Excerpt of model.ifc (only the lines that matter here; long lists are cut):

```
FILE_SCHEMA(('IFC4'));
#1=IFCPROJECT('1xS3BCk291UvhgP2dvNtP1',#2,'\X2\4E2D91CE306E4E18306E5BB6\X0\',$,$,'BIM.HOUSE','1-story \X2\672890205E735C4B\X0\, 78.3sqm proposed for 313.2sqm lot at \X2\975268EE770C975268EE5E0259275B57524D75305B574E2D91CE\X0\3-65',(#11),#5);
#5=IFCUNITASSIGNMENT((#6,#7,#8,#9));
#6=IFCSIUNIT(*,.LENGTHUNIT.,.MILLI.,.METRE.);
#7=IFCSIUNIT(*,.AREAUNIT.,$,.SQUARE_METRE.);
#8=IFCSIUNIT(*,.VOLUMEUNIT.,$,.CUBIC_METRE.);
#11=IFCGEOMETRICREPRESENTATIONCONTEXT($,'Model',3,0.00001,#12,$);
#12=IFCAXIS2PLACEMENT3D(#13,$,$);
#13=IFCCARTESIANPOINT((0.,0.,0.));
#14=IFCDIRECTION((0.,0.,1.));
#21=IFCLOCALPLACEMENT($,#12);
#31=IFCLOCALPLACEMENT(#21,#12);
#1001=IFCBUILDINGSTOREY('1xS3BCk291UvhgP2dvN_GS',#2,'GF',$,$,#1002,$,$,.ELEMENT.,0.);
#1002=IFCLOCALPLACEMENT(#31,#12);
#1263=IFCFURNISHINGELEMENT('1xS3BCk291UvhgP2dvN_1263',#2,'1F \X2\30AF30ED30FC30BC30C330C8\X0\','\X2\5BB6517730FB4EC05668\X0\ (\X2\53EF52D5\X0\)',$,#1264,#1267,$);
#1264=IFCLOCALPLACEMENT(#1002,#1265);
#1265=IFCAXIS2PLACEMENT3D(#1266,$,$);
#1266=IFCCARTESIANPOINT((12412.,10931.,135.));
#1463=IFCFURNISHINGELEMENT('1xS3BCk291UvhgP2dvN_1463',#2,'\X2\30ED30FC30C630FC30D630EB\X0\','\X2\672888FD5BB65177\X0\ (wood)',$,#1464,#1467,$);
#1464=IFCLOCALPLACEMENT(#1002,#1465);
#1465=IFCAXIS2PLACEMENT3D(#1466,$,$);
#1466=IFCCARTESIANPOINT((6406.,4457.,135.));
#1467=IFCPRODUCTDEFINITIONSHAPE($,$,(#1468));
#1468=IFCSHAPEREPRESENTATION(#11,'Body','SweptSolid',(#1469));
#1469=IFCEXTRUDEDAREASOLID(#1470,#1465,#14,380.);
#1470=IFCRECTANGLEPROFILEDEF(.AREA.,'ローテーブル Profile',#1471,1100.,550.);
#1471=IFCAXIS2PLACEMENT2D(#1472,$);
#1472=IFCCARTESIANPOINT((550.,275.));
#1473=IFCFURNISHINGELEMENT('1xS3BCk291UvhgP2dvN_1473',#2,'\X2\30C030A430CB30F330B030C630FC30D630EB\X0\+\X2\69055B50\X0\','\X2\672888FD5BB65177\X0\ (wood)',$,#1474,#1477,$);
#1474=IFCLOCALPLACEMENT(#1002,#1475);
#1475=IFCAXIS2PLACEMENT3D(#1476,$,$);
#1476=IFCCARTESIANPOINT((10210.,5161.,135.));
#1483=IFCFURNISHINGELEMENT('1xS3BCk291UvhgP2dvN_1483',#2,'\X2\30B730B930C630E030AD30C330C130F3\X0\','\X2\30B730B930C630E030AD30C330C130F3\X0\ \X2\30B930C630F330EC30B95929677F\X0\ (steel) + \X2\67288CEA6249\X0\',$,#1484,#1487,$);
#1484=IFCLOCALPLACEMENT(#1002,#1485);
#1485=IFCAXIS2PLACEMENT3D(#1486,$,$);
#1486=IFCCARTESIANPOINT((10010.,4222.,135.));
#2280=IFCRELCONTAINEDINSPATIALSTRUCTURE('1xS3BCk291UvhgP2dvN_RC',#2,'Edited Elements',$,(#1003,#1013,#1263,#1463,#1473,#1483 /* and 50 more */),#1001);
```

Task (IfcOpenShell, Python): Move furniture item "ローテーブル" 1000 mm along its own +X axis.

```python
import ifcopenshell
import ifcopenshell.api.geometry
import ifcopenshell.util.placement

model = ifcopenshell.open("model.ifc")

item = model.by_guid("1xS3BCk291UvhgP2dvN_1463")
matrix = ifcopenshell.util.placement.get_local_placement(item.ObjectPlacement)
matrix[:3, 3] += matrix[:3, 0] * 1000.0
ifcopenshell.api.geometry.edit_object_placement(model, product=item, matrix=matrix, is_si=False)

print(ifcopenshell.util.placement.get_local_placement(item.ObjectPlacement).round(3) + 0.0)

model.write("model-out.ifc")
```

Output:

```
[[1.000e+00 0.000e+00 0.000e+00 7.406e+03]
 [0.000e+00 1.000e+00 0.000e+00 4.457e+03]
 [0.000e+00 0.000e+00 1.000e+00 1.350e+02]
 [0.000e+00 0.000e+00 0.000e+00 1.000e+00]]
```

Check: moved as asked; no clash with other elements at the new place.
